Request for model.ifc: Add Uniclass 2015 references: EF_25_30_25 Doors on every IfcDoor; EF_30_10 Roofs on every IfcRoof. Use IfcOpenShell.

First a look at what the model holds.

```python
import ifcopenshell

model = ifcopenshell.open("model.ifc")
print(model.schema)
print("classifications:", [c.Name for c in model.by_type("IfcClassification")])
for ifc_class in ("IfcDoor", "IfcRoof", "IfcStair", "IfcWall", "IfcWindow"):
    print(ifc_class, len(model.by_type(ifc_class)))
```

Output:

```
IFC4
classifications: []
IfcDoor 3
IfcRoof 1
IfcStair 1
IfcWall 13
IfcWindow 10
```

```python
import ifcopenshell
import ifcopenshell.api.classification

model = ifcopenshell.open("model.ifc")

system = ifcopenshell.api.classification.add_classification(model, classification="Uniclass 2015")

codes = {
    "IfcDoor": ("EF_25_30_25", "Doors"),
    "IfcRoof": ("EF_30_10", "Roofs"),
}
for ifc_class, (code, name) in codes.items():
    products = model.by_type(ifc_class)
    ifcopenshell.api.classification.add_reference(
        model, products=products, classification=system, identification=code, name=name
    )
    print(code, len(products))

model.write("model-out.ifc")
```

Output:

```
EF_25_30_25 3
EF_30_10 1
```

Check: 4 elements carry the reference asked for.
